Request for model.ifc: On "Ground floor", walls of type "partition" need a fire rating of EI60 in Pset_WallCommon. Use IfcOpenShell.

First a look at what the model holds.

```python
import ifcopenshell
import ifcopenshell.util.element

model = ifcopenshell.open("model.ifc")
print(model.schema)
storey = next(s for s in model.by_type("IfcBuildingStorey") if s.Name == "Ground floor")
walls = [e for e in ifcopenshell.util.element.get_decomposition(storey) if e.is_a("IfcWall")]
seen = {}
for e in walls:
    element_type = ifcopenshell.util.element.get_type(e)
    key = (element_type.Name if element_type != e and element_type else None, ifcopenshell.util.element.get_pset(e, "Pset_WallCommon", "FireRating"))
    seen[key] = seen.get(key, 0) + 1
for (name, value), count in sorted(seen.items(), key=str):
    print(count, "x", name, "|", value)
```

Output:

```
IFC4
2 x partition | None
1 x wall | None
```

```python
import ifcopenshell
import ifcopenshell.api.pset
import ifcopenshell.util.element

model = ifcopenshell.open("model.ifc")

storey = next(s for s in model.by_type("IfcBuildingStorey") if s.Name == "Ground floor")
walls = [e for e in ifcopenshell.util.element.get_decomposition(storey) if e.is_a("IfcWall")]

count = 0
for e in walls:
    element_type = ifcopenshell.util.element.get_type(e)
    if element_type in (None, e) or element_type.Name != "partition":
        continue
    # add_pset returns the element's existing set when there is one.
    pset = ifcopenshell.api.pset.add_pset(model, product=e, name="Pset_WallCommon")
    ifcopenshell.api.pset.edit_pset(model, pset=pset, properties={"FireRating": "EI60"})
    count += 1

print(count, "walls updated")

model.write("model-out.ifc")
```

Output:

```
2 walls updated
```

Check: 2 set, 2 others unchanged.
